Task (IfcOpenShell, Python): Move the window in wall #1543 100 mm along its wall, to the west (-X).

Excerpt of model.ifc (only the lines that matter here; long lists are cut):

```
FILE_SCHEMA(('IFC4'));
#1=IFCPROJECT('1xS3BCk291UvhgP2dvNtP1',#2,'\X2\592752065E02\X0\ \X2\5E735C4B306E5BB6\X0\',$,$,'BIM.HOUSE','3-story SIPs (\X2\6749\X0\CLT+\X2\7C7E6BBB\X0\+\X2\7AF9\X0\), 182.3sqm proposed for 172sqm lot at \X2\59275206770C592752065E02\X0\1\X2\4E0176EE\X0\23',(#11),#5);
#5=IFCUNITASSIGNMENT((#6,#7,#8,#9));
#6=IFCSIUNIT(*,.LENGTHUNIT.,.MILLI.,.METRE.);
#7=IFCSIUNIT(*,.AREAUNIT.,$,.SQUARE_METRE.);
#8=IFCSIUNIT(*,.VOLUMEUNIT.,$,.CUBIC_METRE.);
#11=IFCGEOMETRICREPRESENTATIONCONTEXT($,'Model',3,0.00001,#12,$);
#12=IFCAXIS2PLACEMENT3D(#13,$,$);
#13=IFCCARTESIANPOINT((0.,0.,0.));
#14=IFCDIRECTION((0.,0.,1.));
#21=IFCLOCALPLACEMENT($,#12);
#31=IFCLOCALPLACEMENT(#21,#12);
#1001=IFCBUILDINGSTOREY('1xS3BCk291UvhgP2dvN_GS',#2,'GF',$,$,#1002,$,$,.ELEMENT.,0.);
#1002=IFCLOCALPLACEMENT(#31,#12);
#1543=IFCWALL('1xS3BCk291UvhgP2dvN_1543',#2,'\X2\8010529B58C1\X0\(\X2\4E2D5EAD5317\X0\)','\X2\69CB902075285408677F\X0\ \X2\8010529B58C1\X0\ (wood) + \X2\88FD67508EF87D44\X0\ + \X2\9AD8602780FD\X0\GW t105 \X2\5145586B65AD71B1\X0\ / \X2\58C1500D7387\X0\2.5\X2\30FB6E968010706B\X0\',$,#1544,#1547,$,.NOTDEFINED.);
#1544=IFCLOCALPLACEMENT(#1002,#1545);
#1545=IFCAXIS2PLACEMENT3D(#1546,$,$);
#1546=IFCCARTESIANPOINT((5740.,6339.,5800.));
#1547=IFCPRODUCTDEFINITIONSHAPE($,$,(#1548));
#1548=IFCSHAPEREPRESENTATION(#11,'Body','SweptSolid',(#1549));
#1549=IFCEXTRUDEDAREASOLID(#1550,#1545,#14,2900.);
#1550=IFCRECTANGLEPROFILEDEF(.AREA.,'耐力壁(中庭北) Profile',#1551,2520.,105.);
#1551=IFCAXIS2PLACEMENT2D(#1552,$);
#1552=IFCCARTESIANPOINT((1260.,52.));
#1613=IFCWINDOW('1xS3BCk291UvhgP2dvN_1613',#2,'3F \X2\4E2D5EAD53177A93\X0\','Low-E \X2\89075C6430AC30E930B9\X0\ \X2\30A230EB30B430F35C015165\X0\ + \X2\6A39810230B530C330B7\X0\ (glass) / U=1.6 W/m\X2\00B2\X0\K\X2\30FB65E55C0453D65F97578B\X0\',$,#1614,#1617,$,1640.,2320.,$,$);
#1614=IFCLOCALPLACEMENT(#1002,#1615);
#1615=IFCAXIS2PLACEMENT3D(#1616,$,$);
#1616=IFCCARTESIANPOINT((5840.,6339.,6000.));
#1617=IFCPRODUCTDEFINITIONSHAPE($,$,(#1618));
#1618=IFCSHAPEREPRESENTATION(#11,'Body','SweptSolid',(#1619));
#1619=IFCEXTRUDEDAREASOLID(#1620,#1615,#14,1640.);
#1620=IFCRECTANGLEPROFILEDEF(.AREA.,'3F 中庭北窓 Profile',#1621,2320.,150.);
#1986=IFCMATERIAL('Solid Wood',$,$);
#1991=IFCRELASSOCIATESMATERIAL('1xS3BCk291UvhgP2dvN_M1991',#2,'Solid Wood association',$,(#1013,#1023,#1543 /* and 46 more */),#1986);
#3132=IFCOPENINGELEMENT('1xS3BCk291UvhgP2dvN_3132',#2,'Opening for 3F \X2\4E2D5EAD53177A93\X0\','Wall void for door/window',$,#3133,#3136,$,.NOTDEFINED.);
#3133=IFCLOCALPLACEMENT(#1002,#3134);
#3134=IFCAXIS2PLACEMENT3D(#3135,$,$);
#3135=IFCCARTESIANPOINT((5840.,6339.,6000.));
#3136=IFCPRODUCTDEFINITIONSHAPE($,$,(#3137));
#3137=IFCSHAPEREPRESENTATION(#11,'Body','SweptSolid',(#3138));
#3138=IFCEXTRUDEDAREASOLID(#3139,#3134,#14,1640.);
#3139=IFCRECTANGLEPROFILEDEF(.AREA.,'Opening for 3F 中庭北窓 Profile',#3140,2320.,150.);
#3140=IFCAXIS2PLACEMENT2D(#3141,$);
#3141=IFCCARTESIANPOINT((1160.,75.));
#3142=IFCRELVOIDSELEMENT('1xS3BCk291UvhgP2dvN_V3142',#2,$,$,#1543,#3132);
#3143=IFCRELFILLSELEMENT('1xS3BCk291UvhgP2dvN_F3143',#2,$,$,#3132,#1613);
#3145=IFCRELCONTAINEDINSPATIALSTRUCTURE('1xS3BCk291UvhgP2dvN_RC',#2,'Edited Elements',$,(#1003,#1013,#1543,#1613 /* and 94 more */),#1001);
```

```python
import ifcopenshell
import ifcopenshell.api.geometry
import ifcopenshell.util.placement
import ifcopenshell.util.unit

model = ifcopenshell.open("model.ifc")
unit_scale = ifcopenshell.util.unit.calculate_unit_scale(model)

window = model.by_id(1613)
opening = window.FillsVoids[0].RelatingOpeningElement
wall = opening.VoidsElements[0].RelatingBuildingElement

wall_matrix = ifcopenshell.util.placement.get_local_placement(wall.ObjectPlacement)
shift = wall_matrix[:3, 0] * -0.1 / unit_scale
before = ifcopenshell.util.placement.get_local_placement(window.ObjectPlacement)[:3, 3].copy()

# The window is not placed relative to its opening, so move both.
for product in (opening, window):
    matrix = ifcopenshell.util.placement.get_local_placement(product.ObjectPlacement)
    matrix[:3, 3] += shift
    ifcopenshell.api.geometry.edit_object_placement(model, product=product, matrix=matrix, is_si=False)

after = ifcopenshell.util.placement.get_local_placement(window.ObjectPlacement)[:3, 3]
print("window moved by", (after - before).round(3) + 0.0)

model.write("model_updated.ifc")
```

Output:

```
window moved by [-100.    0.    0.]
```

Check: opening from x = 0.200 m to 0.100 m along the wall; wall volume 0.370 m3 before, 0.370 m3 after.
